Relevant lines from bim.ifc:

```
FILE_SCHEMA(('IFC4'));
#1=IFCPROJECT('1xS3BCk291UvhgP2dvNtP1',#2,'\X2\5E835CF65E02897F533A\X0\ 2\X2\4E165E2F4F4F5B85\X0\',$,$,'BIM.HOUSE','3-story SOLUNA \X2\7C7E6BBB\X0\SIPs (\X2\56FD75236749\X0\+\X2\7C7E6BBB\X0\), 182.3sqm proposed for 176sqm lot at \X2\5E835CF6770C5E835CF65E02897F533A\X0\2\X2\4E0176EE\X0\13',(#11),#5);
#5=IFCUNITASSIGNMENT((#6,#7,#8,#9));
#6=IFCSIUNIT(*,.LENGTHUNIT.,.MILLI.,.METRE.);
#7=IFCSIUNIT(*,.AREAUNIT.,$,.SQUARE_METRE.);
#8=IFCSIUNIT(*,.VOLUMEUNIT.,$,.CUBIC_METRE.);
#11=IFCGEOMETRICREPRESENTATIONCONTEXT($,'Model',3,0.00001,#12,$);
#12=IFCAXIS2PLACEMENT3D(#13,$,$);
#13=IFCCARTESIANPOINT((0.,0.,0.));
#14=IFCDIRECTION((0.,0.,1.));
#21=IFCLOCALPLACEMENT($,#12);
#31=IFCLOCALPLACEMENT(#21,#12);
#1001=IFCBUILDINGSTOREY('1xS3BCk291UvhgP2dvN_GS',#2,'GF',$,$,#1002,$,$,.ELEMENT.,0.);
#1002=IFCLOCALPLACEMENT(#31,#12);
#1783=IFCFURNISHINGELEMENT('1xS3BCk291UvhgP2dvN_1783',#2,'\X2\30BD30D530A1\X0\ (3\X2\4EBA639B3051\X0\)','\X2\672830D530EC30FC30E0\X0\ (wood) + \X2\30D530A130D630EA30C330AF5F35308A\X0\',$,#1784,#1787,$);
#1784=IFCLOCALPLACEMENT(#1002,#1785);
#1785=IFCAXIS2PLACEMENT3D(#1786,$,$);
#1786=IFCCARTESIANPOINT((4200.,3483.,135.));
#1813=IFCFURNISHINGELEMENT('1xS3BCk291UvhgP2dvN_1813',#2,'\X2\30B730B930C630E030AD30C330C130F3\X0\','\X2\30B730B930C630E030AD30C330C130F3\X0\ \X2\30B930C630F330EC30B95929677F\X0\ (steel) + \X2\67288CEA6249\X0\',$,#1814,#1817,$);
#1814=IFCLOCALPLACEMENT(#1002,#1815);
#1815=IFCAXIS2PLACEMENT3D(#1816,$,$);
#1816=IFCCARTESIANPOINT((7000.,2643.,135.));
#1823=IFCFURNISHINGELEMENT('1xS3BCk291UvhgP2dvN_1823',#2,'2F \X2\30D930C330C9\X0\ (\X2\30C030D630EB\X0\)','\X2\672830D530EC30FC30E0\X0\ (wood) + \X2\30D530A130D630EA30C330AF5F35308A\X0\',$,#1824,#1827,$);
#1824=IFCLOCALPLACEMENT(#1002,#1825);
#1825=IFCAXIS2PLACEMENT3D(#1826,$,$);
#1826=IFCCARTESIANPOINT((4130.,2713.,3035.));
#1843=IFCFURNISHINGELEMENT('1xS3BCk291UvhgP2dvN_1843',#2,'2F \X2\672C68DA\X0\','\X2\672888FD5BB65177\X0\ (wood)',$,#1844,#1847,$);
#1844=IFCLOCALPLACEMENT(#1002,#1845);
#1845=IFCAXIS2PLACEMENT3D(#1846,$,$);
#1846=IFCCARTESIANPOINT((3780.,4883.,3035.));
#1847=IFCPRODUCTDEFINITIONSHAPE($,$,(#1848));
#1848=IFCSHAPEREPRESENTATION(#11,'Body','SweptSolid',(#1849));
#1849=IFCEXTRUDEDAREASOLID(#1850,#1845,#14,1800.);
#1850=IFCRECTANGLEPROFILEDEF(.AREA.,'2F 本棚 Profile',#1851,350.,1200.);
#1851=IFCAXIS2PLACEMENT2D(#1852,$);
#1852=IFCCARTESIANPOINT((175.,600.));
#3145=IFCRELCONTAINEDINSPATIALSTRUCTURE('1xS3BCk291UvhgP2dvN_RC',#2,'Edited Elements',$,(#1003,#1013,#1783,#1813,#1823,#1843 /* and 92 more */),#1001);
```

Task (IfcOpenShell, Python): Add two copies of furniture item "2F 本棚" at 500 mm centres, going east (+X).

```python
import numpy as np
import ifcopenshell
import ifcopenshell.api.geometry
import ifcopenshell.api.root
import ifcopenshell.util.element
import ifcopenshell.util.placement
import ifcopenshell.util.unit

model = ifcopenshell.open("bim.ifc")
unit_scale = ifcopenshell.util.unit.calculate_unit_scale(model)


def reuse_history(source, copy):
    """copy_class also copies each property set's owner history, people and application; keep the originals."""
    for rel in copy.IsDefinedBy:
        if rel.is_a("IfcRelDefinesByProperties") and (history := rel.RelatingPropertyDefinition.OwnerHistory):
            rel.RelatingPropertyDefinition.OwnerHistory = source.OwnerHistory
            ifcopenshell.util.element.remove_deep2(model, history)


source = model.by_id(1843)
base = ifcopenshell.util.placement.get_local_placement(source.ObjectPlacement)
step = np.array([1.0, 0.0, 0.0]) * 0.5 / unit_scale

for i in range(1, 3):
    copy = ifcopenshell.api.root.copy_class(model, product=source)
    copy.Representation = ifcopenshell.util.element.copy_deep(
        model, source.Representation, exclude=["IfcGeometricRepresentationContext", "IfcRepresentationMap"]
    )
    reuse_history(source, copy)
    matrix = base.copy()
    matrix[:3, 3] += i * step
    print("added at", matrix[:3, 3].round(3) + 0.0)
    ifcopenshell.api.geometry.edit_object_placement(model, product=copy, matrix=matrix, is_si=False)

model.write("bim_rev.ifc")
```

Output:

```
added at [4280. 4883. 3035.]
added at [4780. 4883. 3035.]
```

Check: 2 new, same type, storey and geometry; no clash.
